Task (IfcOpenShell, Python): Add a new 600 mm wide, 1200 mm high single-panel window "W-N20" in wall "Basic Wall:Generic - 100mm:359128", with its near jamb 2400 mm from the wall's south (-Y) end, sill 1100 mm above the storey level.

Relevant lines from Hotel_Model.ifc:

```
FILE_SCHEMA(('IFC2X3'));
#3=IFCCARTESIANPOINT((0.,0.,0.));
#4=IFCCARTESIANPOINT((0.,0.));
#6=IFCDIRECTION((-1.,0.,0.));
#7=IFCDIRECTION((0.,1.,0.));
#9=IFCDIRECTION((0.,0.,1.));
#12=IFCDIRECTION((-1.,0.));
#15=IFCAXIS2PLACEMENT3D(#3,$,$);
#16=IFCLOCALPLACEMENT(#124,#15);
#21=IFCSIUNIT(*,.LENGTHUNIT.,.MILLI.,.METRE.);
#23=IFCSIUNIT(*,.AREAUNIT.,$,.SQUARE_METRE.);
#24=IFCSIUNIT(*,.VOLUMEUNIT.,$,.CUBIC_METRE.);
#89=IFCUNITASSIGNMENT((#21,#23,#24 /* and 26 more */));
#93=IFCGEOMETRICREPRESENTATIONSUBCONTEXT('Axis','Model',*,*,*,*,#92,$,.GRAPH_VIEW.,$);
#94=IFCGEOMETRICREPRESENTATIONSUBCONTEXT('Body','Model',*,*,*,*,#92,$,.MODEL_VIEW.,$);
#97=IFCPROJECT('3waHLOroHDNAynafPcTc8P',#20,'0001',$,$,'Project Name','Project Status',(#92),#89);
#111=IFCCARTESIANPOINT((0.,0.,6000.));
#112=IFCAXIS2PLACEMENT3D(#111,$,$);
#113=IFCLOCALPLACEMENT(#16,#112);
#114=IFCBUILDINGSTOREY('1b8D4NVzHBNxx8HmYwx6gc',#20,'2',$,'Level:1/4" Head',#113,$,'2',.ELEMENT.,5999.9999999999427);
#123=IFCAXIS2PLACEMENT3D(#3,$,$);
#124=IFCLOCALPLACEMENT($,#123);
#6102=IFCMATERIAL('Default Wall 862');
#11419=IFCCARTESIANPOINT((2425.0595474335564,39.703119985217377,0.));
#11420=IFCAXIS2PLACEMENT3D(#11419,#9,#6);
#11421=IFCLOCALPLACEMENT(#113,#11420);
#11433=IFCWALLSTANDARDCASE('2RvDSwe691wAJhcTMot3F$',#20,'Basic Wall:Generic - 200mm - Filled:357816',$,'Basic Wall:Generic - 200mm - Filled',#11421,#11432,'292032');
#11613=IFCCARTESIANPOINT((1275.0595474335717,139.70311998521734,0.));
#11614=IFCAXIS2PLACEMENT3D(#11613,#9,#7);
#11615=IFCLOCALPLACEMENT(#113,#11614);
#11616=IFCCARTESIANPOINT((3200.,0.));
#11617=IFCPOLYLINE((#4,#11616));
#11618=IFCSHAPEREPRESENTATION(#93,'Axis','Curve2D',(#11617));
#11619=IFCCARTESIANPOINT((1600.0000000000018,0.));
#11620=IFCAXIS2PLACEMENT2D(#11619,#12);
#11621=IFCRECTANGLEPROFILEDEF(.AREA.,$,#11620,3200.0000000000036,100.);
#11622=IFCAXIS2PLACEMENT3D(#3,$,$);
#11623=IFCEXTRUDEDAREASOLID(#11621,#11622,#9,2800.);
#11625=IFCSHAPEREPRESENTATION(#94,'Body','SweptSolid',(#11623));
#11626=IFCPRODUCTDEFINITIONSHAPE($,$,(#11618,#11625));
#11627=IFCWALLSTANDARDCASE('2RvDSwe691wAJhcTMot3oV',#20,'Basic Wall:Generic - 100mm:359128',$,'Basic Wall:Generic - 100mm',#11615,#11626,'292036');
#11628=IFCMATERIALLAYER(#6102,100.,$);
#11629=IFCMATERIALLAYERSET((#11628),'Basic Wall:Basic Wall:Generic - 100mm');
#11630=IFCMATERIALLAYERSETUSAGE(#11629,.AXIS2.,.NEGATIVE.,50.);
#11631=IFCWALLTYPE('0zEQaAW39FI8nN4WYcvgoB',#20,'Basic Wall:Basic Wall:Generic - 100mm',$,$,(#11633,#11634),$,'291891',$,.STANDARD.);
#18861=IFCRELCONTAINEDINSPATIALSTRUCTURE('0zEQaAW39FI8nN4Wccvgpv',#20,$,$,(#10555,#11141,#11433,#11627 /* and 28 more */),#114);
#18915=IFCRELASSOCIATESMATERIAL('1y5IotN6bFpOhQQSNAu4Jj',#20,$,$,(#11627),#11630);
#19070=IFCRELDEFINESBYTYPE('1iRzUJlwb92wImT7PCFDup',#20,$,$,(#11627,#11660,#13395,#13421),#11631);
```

```python
import numpy as np
import ifcopenshell
import ifcopenshell.api.feature
import ifcopenshell.api.geometry
import ifcopenshell.api.root
import ifcopenshell.api.spatial
import ifcopenshell.api.type
import ifcopenshell.geom
import ifcopenshell.util.element
import ifcopenshell.util.placement
import ifcopenshell.util.representation
import ifcopenshell.util.shape
import ifcopenshell.util.unit

model = ifcopenshell.open("Hotel_Model.ifc")
unit_scale = ifcopenshell.util.unit.calculate_unit_scale(model)
settings = ifcopenshell.geom.settings()


def volume(element):
    """Net volume in cubic metres, openings subtracted."""
    shape = ifcopenshell.geom.create_shape(settings, element)
    return ifcopenshell.util.shape.get_volume(shape.geometry)


wall = model.by_guid("2RvDSwe691wAJhcTMot3oV")
storey = ifcopenshell.util.element.get_container(wall, ifc_class="IfcBuildingStorey")
context = ifcopenshell.util.representation.get_context(model, "Model", "Body", "MODEL_VIEW")
before = volume(wall)

width, height, from_end, sill = 0.6, 1.2, 2.4, 1.1  # metres

# The wall runs along its own X axis, and the end named is its -X end.
wall_shape = ifcopenshell.geom.create_shape(settings, wall)
x, y, z = ifcopenshell.util.shape.get_vertices(wall_shape.geometry).T
start = x.min() + from_end
face, thickness = float(y.min()), float(y.max() - y.min())
wall_matrix = ifcopenshell.util.placement.get_local_placement(wall.ObjectPlacement)
level = ifcopenshell.util.placement.get_local_placement(storey.ObjectPlacement)[2, 3]


def in_wall(x, y):
    """Placement at x, y metres in the wall's axes, at sill height."""
    matrix = wall_matrix.copy()
    matrix[:, 3] = wall_matrix @ np.array([x / unit_scale, y / unit_scale, 0.0, 1.0])
    matrix[2, 3] = level + sill / unit_scale
    return matrix


# Opening: a box that overshoots both wall faces by 50 mm.
opening = ifcopenshell.api.root.create_entity(model, ifc_class="IfcOpeningElement")
box = ifcopenshell.api.geometry.add_wall_representation(
    model, context=context, length=width, height=height, thickness=thickness + 0.1
)
ifcopenshell.api.geometry.assign_representation(model, product=opening, representation=box)
ifcopenshell.api.geometry.edit_object_placement(model, product=opening, matrix=in_wall(start, face - 0.05), is_si=False)
ifcopenshell.api.feature.add_feature(model, feature=opening, element=wall)

window = ifcopenshell.api.root.create_entity(model, ifc_class="IfcWindow", name="W-N20")
window.OverallWidth, window.OverallHeight = width / unit_scale, height / unit_scale
body = ifcopenshell.api.geometry.add_window_representation(
    model,
    context=context,
    overall_width=window.OverallWidth,
    overall_height=window.OverallHeight,
    partition_type="SINGLE_PANEL",
)
ifcopenshell.api.geometry.assign_representation(model, product=window, representation=body)
ifcopenshell.api.spatial.assign_container(model, products=[window], relating_structure=storey)
fills = ifcopenshell.api.feature.add_filling(model, opening=opening, element=window)
fills.OwnerHistory = window.OwnerHistory  # required in IFC2X3

# IFC2X3 keeps the operation on the window style.
style = ifcopenshell.api.root.create_entity(model, ifc_class="IfcWindowStyle", name="W-N20")
style.OperationType, style.ConstructionType = "SINGLE_PANEL", "NOTDEFINED"
style.ParameterTakesPrecedence = style.Sizeable = False
ifcopenshell.api.type.assign_type(model, related_objects=[window], relating_type=style)

# Centre the window in the wall's thickness.
ifcopenshell.api.geometry.edit_object_placement(model, product=window, matrix=in_wall(start, face), is_si=False)
window_shape = ifcopenshell.geom.create_shape(settings, window)
depth = ifcopenshell.util.shape.get_vertices(window_shape.geometry)[:, 1]
offset = face + thickness / 2 - (depth.min() + depth.max()) / 2
ifcopenshell.api.geometry.edit_object_placement(model, product=window, matrix=in_wall(start, offset), is_si=False)

after = volume(wall)

print(f"wall volume {before:.3f} -> {after:.3f} m3")

model.write("Hotel_Model_v2.ifc")
```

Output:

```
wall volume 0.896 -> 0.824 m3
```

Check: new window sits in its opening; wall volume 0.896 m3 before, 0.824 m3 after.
